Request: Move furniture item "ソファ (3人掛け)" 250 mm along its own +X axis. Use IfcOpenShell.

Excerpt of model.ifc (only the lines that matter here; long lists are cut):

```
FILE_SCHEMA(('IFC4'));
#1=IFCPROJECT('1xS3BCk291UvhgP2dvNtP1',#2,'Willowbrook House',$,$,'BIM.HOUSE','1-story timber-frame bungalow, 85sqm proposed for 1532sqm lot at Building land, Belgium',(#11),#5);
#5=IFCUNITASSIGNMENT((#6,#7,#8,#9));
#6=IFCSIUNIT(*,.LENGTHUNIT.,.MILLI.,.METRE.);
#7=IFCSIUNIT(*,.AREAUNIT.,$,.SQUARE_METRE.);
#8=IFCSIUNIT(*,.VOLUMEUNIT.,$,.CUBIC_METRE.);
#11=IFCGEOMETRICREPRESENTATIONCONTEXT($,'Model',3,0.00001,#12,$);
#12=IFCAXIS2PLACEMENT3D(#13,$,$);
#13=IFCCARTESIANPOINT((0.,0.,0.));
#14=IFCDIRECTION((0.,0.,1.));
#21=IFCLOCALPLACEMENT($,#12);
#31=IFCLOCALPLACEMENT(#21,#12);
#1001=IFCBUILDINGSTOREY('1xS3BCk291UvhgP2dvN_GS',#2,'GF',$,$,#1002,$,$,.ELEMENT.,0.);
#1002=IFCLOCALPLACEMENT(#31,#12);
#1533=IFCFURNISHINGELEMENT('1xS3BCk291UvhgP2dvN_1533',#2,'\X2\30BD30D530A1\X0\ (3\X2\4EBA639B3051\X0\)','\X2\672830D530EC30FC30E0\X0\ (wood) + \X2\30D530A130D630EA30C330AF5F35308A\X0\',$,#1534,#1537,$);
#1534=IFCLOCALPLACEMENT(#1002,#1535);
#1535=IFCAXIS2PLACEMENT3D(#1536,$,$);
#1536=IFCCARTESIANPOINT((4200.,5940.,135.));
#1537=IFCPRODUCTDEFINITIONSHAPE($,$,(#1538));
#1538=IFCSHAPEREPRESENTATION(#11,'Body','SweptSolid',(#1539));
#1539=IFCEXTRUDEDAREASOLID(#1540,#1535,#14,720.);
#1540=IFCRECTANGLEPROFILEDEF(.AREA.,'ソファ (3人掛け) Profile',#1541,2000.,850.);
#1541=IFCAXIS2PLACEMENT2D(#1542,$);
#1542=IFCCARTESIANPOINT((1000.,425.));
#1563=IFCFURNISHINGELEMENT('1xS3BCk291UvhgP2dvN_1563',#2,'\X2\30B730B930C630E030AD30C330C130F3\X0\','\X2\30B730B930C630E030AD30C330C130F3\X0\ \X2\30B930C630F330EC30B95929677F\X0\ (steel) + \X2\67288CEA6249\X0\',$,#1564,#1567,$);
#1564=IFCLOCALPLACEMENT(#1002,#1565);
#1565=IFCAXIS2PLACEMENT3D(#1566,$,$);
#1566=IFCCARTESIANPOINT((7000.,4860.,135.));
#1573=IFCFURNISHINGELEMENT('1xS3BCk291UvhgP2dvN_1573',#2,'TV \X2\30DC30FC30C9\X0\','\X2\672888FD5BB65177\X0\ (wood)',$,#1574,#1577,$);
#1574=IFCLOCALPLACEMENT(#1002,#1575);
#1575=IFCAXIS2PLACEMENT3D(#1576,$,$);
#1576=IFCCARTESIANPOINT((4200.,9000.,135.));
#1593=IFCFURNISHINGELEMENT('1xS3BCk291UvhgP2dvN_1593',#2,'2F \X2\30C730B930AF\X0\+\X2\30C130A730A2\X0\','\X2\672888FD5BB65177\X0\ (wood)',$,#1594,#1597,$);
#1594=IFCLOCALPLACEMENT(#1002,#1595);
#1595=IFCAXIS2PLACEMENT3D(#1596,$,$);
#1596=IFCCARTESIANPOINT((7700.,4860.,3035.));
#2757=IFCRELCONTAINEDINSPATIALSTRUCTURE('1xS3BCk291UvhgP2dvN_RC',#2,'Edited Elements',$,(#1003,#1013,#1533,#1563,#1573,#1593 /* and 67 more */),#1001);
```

```python
import ifcopenshell
import ifcopenshell.api.geometry
import ifcopenshell.util.placement
import ifcopenshell.util.unit

model = ifcopenshell.open("model.ifc")
unit_scale = ifcopenshell.util.unit.calculate_unit_scale(model)

item = model.by_guid("1xS3BCk291UvhgP2dvN_1533")
matrix = ifcopenshell.util.placement.get_local_placement(item.ObjectPlacement)
matrix[:3, 3] += matrix[:3, 0] * 0.25 / unit_scale
ifcopenshell.api.geometry.edit_object_placement(model, product=item, matrix=matrix, is_si=False)

print(ifcopenshell.util.placement.get_local_placement(item.ObjectPlacement).round(3) + 0.0)

model.write("model_edited.ifc")
```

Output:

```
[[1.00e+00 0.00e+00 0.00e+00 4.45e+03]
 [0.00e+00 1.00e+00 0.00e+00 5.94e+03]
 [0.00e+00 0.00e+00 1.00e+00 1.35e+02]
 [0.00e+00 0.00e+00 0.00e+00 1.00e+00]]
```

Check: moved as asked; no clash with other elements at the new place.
